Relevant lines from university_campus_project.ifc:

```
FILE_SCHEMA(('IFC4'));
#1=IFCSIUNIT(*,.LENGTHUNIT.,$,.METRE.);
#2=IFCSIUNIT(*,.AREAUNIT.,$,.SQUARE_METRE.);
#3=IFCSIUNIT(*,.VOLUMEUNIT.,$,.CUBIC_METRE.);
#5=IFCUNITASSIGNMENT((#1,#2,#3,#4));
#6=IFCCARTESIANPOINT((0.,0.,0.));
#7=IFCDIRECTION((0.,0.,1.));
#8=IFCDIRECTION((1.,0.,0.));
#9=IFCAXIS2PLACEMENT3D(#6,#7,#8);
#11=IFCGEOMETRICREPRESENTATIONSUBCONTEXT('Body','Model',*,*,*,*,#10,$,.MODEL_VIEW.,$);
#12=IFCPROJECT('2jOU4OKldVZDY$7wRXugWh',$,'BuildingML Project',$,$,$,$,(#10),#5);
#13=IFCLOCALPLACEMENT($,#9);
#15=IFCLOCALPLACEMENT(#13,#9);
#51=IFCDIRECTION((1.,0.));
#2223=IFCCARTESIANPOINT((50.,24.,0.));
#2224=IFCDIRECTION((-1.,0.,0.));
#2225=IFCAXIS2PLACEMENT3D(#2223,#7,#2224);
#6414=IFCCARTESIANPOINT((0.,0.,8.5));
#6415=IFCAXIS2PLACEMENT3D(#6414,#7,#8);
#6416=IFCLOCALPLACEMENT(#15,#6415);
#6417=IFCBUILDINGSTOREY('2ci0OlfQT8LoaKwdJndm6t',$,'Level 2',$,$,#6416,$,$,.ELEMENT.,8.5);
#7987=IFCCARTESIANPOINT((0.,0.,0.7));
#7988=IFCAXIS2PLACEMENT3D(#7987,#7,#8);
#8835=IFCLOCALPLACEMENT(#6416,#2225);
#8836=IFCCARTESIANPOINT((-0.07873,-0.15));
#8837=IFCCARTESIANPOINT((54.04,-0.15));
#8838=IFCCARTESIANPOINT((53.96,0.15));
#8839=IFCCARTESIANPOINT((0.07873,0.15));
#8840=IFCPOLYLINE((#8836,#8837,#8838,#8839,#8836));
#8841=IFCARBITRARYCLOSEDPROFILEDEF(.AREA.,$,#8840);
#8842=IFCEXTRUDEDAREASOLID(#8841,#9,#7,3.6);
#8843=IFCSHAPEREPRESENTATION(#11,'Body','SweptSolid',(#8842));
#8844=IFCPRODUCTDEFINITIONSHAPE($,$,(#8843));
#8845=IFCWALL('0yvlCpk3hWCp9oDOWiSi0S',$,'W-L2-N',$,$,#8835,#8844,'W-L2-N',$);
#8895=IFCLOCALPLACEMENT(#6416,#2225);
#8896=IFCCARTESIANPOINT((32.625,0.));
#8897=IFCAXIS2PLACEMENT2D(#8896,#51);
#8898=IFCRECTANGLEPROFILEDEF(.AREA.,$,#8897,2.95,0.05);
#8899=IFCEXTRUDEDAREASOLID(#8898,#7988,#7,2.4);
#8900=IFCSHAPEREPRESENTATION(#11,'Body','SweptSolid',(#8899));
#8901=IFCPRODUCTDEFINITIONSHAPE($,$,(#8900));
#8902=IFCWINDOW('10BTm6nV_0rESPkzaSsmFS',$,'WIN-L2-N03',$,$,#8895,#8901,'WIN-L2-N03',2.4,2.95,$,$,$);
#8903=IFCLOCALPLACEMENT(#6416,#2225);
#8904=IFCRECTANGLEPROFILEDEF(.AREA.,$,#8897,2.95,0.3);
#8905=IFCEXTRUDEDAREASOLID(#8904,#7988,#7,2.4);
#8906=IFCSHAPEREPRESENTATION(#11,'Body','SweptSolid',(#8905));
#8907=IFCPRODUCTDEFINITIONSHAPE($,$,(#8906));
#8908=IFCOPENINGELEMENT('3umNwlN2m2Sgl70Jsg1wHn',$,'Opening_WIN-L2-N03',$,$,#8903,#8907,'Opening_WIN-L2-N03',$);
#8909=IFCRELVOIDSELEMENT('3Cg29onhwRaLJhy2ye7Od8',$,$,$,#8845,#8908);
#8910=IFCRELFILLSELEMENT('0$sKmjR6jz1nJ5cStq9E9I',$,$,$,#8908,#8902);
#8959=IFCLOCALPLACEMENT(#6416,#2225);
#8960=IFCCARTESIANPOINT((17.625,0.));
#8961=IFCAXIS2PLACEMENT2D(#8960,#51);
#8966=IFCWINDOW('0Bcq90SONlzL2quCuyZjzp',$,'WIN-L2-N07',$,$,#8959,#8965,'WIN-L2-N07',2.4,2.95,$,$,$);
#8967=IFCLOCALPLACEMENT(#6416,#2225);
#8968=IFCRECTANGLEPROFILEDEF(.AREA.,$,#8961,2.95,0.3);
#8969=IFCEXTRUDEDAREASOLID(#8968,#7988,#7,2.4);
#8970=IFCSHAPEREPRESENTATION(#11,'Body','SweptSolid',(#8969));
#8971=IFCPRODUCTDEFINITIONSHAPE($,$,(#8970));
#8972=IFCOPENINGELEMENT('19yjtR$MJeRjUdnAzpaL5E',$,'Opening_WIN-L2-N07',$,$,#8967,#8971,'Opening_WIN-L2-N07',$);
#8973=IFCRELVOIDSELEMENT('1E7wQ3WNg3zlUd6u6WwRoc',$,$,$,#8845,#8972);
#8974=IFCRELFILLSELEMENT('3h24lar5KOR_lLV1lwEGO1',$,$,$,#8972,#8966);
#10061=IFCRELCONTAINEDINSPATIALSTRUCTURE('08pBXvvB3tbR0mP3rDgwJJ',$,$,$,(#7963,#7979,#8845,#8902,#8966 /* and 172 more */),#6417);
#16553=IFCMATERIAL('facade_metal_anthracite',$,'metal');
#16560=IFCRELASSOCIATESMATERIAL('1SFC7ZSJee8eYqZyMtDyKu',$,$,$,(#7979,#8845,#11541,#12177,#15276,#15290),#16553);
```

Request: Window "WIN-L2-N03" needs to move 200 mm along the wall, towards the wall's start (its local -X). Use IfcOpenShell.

```python
import ifcopenshell
import ifcopenshell.api.geometry
import ifcopenshell.util.placement
import ifcopenshell.util.unit

model = ifcopenshell.open("university_campus_project.ifc")
unit_scale = ifcopenshell.util.unit.calculate_unit_scale(model)

window = model.by_id(8902)
opening = window.FillsVoids[0].RelatingOpeningElement
wall = opening.VoidsElements[0].RelatingBuildingElement

wall_matrix = ifcopenshell.util.placement.get_local_placement(wall.ObjectPlacement)
shift = wall_matrix[:3, 0] * -0.2 / unit_scale
before = ifcopenshell.util.placement.get_local_placement(window.ObjectPlacement)[:3, 3].copy()

# The window is not placed relative to its opening, so move both.
for product in (opening, window):
    matrix = ifcopenshell.util.placement.get_local_placement(product.ObjectPlacement)
    matrix[:3, 3] += shift
    ifcopenshell.api.geometry.edit_object_placement(model, product=product, matrix=matrix, is_si=False)

after = ifcopenshell.util.placement.get_local_placement(window.ObjectPlacement)[:3, 3]
print("window moved by", (after - before).round(3) + 0.0)

model.write("university_campus_project_edited.ifc")
```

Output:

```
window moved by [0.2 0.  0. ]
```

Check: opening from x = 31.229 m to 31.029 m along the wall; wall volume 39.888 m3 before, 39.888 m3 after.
